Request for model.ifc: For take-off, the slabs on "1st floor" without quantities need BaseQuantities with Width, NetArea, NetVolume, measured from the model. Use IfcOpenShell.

First a look at what the model holds.

```python
import ifcopenshell
import ifcopenshell.util.element
import ifcopenshell.util.unit

model = ifcopenshell.open("model.ifc")
print(model.schema)
for unit_type in ("LENGTHUNIT", "AREAUNIT", "VOLUMEUNIT"):
    print(unit_type, ifcopenshell.util.unit.calculate_unit_scale(model, unit_type))
storey = next(s for s in model.by_type("IfcBuildingStorey") if s.Name == "1st floor")
slabs = [e for e in ifcopenshell.util.element.get_decomposition(storey) if e.is_a("IfcSlab")]
for e in sorted(slabs, key=lambda e: e.id()):
    print(e.id(), e.is_a(), e.Name, list(ifcopenshell.util.element.get_psets(e, qtos_only=True)), sep=" | ")
```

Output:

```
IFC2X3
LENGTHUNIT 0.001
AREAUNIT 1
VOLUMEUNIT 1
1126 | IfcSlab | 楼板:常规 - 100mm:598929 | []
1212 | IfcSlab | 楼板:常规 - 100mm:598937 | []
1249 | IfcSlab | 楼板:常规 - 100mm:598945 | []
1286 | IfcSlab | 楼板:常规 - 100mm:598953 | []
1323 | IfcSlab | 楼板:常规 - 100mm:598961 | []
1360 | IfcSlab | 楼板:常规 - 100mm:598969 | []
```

```python
import ifcopenshell
import ifcopenshell.api.pset
import ifcopenshell.geom
import ifcopenshell.util.element
import ifcopenshell.util.shape
import ifcopenshell.util.unit

model = ifcopenshell.open("model.ifc")
unit_scale = ifcopenshell.util.unit.calculate_unit_scale(model)
area_scale = ifcopenshell.util.unit.calculate_unit_scale(model, "AREAUNIT")
volume_scale = ifcopenshell.util.unit.calculate_unit_scale(model, "VOLUMEUNIT")
settings = ifcopenshell.geom.settings()

storey = next(s for s in model.by_type("IfcBuildingStorey") if s.Name == "1st floor")
slabs = [e for e in ifcopenshell.util.element.get_decomposition(storey) if e.is_a("IfcSlab")]

for e in sorted(slabs, key=lambda e: e.id()):
    if ifcopenshell.util.element.get_psets(e, qtos_only=True, should_inherit=False):
        continue
    # Geometry comes back in metres, in the element's own axes.
    shape = ifcopenshell.geom.create_shape(settings, e)
    values = {
        "Width": ifcopenshell.util.shape.get_z(shape.geometry) / unit_scale,
        "NetArea": ifcopenshell.util.shape.get_footprint_area(shape.geometry) / area_scale,
        "NetVolume": ifcopenshell.util.shape.get_volume(shape.geometry) / volume_scale,
    }
    qto = ifcopenshell.api.pset.add_qto(model, product=e, name="BaseQuantities")
    ifcopenshell.api.pset.edit_qto(model, qto=qto, properties=values)
    print(e.id(), {k: round(v, 3) for k, v in values.items()})

model.write("model_updated.ifc")
```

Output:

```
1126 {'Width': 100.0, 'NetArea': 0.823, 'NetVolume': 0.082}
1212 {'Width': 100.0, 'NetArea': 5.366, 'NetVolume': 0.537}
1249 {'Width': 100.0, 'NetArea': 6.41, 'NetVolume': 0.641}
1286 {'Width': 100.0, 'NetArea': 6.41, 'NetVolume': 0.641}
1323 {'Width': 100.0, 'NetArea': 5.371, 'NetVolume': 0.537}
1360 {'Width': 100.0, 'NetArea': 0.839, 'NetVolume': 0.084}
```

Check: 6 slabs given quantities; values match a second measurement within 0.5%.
